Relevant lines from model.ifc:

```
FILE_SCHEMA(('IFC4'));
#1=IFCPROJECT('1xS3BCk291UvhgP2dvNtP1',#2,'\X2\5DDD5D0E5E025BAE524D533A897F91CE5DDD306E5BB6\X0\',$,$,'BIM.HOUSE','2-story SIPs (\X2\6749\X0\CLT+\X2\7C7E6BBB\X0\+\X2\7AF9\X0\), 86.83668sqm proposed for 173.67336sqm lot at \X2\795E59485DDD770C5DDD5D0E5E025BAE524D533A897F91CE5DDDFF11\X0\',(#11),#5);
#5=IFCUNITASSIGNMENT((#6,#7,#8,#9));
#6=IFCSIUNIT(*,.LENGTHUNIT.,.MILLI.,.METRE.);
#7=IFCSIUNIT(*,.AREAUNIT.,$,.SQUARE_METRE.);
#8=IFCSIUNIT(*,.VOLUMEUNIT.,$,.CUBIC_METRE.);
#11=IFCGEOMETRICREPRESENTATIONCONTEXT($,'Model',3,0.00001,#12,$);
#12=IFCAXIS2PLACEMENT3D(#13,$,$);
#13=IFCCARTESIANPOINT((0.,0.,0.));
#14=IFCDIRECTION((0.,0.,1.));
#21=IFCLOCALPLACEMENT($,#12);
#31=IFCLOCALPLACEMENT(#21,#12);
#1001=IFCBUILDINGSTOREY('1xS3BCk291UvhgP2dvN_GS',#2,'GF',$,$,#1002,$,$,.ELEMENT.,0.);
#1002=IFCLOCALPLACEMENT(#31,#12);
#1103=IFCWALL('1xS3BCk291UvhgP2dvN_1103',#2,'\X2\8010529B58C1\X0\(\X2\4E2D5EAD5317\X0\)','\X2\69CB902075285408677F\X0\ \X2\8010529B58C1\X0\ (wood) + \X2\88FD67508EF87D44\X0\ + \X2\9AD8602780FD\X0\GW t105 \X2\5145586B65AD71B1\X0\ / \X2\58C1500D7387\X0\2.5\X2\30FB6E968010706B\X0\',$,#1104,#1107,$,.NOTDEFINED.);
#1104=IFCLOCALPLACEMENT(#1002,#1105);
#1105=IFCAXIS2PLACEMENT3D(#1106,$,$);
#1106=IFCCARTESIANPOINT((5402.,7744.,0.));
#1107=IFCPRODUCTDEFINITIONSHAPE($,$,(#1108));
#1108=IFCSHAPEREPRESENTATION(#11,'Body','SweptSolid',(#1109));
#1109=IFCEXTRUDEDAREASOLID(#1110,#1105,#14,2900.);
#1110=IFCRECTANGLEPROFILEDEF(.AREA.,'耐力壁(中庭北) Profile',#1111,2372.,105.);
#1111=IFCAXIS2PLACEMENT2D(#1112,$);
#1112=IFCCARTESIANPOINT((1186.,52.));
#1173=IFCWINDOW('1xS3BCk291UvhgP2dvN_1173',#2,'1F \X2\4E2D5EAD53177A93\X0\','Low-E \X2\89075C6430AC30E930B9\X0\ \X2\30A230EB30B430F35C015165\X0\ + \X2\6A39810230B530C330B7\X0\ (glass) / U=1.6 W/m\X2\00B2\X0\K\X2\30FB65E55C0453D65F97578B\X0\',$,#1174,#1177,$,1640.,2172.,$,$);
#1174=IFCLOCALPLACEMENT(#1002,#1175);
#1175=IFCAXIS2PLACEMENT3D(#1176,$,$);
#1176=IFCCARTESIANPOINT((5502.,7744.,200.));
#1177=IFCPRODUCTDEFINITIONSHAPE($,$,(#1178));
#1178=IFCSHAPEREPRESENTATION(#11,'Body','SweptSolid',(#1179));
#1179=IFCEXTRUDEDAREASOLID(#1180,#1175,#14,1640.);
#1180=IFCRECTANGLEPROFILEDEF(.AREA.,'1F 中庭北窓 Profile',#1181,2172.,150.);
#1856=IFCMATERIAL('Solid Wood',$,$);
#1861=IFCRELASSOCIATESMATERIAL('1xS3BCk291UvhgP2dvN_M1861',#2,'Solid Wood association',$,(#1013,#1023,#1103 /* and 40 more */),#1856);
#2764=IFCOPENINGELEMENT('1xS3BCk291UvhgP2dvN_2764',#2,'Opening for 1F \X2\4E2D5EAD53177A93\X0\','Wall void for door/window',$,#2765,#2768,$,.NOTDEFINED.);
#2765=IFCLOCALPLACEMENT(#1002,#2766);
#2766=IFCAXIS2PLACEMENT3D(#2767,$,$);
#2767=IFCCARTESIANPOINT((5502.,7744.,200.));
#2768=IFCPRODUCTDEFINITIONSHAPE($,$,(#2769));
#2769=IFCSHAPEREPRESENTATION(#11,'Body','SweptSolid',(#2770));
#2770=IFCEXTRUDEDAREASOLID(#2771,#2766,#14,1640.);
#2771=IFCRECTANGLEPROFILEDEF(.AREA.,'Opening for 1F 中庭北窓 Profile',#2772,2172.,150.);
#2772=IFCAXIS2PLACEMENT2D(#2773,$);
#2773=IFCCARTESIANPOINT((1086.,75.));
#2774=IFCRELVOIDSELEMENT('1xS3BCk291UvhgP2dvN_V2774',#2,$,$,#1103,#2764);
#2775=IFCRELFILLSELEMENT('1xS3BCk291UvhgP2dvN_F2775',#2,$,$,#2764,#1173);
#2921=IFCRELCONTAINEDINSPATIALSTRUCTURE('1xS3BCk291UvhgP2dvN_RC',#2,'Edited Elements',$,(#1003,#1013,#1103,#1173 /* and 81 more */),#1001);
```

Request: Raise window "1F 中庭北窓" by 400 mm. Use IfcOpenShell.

```python
import numpy as np
import ifcopenshell
import ifcopenshell.api.geometry
import ifcopenshell.util.placement
import ifcopenshell.util.unit

model = ifcopenshell.open("model.ifc")
unit_scale = ifcopenshell.util.unit.calculate_unit_scale(model)

window = model.by_id(1173)
opening = window.FillsVoids[0].RelatingOpeningElement
dz = 0.4 / unit_scale

shift = np.array([0.0, 0.0, dz])
# The window is not placed relative to its opening, so move both.
for product in (opening, window):
    matrix = ifcopenshell.util.placement.get_local_placement(product.ObjectPlacement)
    matrix[:3, 3] += shift
    ifcopenshell.api.geometry.edit_object_placement(model, product=product, matrix=matrix, is_si=False)

print(f"moved by {dz * unit_scale:+.3f} m")

model.write("model_rev.ifc")
```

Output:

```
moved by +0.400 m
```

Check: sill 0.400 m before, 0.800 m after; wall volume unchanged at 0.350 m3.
